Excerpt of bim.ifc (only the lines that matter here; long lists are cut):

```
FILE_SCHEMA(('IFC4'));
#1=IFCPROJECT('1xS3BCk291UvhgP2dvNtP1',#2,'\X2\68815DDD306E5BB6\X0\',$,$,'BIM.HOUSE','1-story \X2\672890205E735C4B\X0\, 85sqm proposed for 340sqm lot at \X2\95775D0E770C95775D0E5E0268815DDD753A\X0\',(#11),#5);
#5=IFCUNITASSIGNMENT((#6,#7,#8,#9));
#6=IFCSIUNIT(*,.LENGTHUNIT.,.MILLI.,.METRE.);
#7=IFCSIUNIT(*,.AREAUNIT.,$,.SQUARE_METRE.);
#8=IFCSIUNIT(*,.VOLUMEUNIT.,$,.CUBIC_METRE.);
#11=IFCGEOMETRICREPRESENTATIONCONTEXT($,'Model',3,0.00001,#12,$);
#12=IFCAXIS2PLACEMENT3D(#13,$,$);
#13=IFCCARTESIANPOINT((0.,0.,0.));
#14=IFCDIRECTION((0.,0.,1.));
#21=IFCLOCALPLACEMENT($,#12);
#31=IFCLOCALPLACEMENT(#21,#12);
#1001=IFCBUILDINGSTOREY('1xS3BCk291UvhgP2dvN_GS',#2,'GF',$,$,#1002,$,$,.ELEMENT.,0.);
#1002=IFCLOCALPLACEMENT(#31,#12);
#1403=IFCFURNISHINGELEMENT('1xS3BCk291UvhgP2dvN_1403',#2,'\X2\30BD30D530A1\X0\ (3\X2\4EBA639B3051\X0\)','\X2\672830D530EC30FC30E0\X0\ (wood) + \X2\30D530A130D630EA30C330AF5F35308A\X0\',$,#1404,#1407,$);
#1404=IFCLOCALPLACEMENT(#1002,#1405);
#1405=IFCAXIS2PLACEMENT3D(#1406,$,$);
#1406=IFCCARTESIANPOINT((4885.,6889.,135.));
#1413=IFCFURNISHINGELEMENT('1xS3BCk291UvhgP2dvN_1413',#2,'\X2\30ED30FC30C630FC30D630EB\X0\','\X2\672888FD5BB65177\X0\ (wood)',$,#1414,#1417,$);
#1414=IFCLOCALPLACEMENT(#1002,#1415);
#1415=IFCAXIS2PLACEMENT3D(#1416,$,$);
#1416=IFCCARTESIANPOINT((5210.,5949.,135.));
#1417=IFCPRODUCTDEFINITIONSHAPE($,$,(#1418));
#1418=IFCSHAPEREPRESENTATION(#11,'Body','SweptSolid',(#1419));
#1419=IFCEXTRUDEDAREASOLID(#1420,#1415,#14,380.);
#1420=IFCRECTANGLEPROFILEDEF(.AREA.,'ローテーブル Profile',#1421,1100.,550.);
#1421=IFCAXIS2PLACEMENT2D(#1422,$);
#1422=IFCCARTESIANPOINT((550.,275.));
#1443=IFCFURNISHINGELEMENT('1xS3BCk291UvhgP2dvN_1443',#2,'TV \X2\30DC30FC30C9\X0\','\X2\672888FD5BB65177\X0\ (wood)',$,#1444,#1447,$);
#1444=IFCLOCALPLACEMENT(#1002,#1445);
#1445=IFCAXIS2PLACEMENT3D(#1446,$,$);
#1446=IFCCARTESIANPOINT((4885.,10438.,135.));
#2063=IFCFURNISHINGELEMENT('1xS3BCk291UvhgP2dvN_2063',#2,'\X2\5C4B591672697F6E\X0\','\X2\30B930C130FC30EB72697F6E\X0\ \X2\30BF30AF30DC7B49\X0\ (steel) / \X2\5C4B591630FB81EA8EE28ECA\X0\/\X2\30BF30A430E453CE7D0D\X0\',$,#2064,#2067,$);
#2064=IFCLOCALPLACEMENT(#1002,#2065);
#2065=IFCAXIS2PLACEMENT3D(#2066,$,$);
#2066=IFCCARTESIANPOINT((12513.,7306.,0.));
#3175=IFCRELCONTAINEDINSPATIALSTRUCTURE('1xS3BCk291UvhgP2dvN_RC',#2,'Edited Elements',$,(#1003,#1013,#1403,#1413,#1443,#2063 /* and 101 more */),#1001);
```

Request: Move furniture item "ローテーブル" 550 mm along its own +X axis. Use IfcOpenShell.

```python
import ifcopenshell
import ifcopenshell.api.geometry
import ifcopenshell.util.placement

model = ifcopenshell.open("bim.ifc")

item = model.by_guid("1xS3BCk291UvhgP2dvN_1413")
matrix = ifcopenshell.util.placement.get_local_placement(item.ObjectPlacement)
matrix[:3, 3] += matrix[:3, 0] * 550.0
ifcopenshell.api.geometry.edit_object_placement(model, product=item, matrix=matrix, is_si=False)

print(ifcopenshell.util.placement.get_local_placement(item.ObjectPlacement).round(3) + 0.0)

model.write("bim_v2.ifc")
```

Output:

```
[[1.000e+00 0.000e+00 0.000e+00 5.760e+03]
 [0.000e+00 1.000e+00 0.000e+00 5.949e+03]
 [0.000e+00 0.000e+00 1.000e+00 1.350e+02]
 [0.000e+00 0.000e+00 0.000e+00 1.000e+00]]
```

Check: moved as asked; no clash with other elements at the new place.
